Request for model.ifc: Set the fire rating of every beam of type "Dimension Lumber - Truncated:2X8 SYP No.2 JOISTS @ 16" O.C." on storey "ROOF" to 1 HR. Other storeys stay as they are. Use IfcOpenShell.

First a look at what the model holds.

```python
import ifcopenshell
import ifcopenshell.util.element

model = ifcopenshell.open("model.ifc")
print(model.schema)
storey = next(s for s in model.by_type("IfcBuildingStorey") if s.Name == "ROOF")
beams = [e for e in ifcopenshell.util.element.get_decomposition(storey) if e.is_a("IfcBeam")]
seen = {}
for e in beams:
    element_type = ifcopenshell.util.element.get_type(e)
    key = (element_type.Name if element_type != e and element_type else None, ifcopenshell.util.element.get_pset(e, "Pset_BeamCommon", "FireRating"))
    seen[key] = seen.get(key, 0) + 1
for (name, value), count in sorted(seen.items(), key=str):
    print(count, "x", name, "|", value)
```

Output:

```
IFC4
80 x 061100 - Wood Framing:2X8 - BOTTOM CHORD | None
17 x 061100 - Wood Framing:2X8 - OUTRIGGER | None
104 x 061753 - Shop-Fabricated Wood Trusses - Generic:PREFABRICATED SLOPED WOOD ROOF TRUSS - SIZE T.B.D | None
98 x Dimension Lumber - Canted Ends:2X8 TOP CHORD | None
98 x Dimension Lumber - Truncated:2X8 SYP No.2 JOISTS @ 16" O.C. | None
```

```python
import ifcopenshell
import ifcopenshell.api.pset
import ifcopenshell.util.element

model = ifcopenshell.open("model.ifc")

storey = next(s for s in model.by_type("IfcBuildingStorey") if s.Name == "ROOF")
beams = [e for e in ifcopenshell.util.element.get_decomposition(storey) if e.is_a("IfcBeam")]

count = 0
for e in beams:
    element_type = ifcopenshell.util.element.get_type(e)
    if element_type in (None, e) or element_type.Name != 'Dimension Lumber - Truncated:2X8 SYP No.2 JOISTS @ 16" O.C.':
        continue
    # add_pset returns the element's existing set when there is one.
    pset = ifcopenshell.api.pset.add_pset(model, product=e, name="Pset_BeamCommon")
    ifcopenshell.api.pset.edit_pset(model, pset=pset, properties={"FireRating": "1 HR"})
    count += 1

print(count, "beams updated")

model.write("model_v2.ifc")
```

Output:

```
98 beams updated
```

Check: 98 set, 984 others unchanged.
